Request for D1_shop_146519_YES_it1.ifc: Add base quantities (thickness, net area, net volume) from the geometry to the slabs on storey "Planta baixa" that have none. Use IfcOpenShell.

First a look at what the model holds.

```python
import ifcopenshell
import ifcopenshell.util.element
import ifcopenshell.util.unit

model = ifcopenshell.open("D1_shop_146519_YES_it1.ifc")
print(model.schema)
for unit_type in ("LENGTHUNIT", "AREAUNIT", "VOLUMEUNIT"):
    print(unit_type, ifcopenshell.util.unit.calculate_unit_scale(model, unit_type))
storey = next(s for s in model.by_type("IfcBuildingStorey") if s.Name == "Planta baixa")
slabs = [e for e in ifcopenshell.util.element.get_decomposition(storey) if e.is_a("IfcSlab")]
for e in sorted(slabs, key=lambda e: e.id()):
    print(e.id(), e.is_a(), e.Name, list(ifcopenshell.util.element.get_psets(e, qtos_only=True)), sep=" | ")
```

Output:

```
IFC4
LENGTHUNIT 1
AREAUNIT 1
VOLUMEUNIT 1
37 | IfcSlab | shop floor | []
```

```python
import ifcopenshell
import ifcopenshell.api.pset
import ifcopenshell.geom
import ifcopenshell.util.element
import ifcopenshell.util.shape
import ifcopenshell.util.unit

model = ifcopenshell.open("D1_shop_146519_YES_it1.ifc")
unit_scale = ifcopenshell.util.unit.calculate_unit_scale(model)
area_scale = ifcopenshell.util.unit.calculate_unit_scale(model, "AREAUNIT")
volume_scale = ifcopenshell.util.unit.calculate_unit_scale(model, "VOLUMEUNIT")
settings = ifcopenshell.geom.settings()

storey = next(s for s in model.by_type("IfcBuildingStorey") if s.Name == "Planta baixa")
slabs = [e for e in ifcopenshell.util.element.get_decomposition(storey) if e.is_a("IfcSlab")]

for e in sorted(slabs, key=lambda e: e.id()):
    if ifcopenshell.util.element.get_psets(e, qtos_only=True, should_inherit=False):
        continue
    # Geometry comes back in metres, in the element's own axes.
    shape = ifcopenshell.geom.create_shape(settings, e)
    values = {
        "Width": ifcopenshell.util.shape.get_z(shape.geometry) / unit_scale,
        "NetArea": ifcopenshell.util.shape.get_footprint_area(shape.geometry) / area_scale,
        "NetVolume": ifcopenshell.util.shape.get_volume(shape.geometry) / volume_scale,
    }
    qto = ifcopenshell.api.pset.add_qto(model, product=e, name="Qto_SlabBaseQuantities")
    ifcopenshell.api.pset.edit_qto(model, qto=qto, properties=values)
    print(e.id(), {k: round(v, 3) for k, v in values.items()})

model.write("D1_shop_146519_YES_it1_v2.ifc")
```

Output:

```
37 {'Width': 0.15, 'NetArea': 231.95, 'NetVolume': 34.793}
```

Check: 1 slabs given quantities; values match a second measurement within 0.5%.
